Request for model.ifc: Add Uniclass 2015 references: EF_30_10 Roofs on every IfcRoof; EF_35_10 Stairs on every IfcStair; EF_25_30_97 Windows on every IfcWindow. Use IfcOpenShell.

First a look at what the model holds.

```python
import ifcopenshell

model = ifcopenshell.open("model.ifc")
print(model.schema)
print("classifications:", [c.Name for c in model.by_type("IfcClassification")])
for ifc_class in ("IfcDoor", "IfcRoof", "IfcStair", "IfcWall", "IfcWindow"):
    print(ifc_class, len(model.by_type(ifc_class)))
```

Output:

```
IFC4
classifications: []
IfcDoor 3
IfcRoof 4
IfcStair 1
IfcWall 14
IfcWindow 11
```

```python
import ifcopenshell
import ifcopenshell.api.classification

model = ifcopenshell.open("model.ifc")

system = ifcopenshell.api.classification.add_classification(model, classification="Uniclass 2015")

codes = {
    "IfcRoof": ("EF_30_10", "Roofs"),
    "IfcStair": ("EF_35_10", "Stairs"),
    "IfcWindow": ("EF_25_30_97", "Windows"),
}
for ifc_class, (code, name) in codes.items():
    products = model.by_type(ifc_class)
    ifcopenshell.api.classification.add_reference(
        model, products=products, classification=system, identification=code, name=name
    )
    print(code, len(products))

model.write("model_rev.ifc")
```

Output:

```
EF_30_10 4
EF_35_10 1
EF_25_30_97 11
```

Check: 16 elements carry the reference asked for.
